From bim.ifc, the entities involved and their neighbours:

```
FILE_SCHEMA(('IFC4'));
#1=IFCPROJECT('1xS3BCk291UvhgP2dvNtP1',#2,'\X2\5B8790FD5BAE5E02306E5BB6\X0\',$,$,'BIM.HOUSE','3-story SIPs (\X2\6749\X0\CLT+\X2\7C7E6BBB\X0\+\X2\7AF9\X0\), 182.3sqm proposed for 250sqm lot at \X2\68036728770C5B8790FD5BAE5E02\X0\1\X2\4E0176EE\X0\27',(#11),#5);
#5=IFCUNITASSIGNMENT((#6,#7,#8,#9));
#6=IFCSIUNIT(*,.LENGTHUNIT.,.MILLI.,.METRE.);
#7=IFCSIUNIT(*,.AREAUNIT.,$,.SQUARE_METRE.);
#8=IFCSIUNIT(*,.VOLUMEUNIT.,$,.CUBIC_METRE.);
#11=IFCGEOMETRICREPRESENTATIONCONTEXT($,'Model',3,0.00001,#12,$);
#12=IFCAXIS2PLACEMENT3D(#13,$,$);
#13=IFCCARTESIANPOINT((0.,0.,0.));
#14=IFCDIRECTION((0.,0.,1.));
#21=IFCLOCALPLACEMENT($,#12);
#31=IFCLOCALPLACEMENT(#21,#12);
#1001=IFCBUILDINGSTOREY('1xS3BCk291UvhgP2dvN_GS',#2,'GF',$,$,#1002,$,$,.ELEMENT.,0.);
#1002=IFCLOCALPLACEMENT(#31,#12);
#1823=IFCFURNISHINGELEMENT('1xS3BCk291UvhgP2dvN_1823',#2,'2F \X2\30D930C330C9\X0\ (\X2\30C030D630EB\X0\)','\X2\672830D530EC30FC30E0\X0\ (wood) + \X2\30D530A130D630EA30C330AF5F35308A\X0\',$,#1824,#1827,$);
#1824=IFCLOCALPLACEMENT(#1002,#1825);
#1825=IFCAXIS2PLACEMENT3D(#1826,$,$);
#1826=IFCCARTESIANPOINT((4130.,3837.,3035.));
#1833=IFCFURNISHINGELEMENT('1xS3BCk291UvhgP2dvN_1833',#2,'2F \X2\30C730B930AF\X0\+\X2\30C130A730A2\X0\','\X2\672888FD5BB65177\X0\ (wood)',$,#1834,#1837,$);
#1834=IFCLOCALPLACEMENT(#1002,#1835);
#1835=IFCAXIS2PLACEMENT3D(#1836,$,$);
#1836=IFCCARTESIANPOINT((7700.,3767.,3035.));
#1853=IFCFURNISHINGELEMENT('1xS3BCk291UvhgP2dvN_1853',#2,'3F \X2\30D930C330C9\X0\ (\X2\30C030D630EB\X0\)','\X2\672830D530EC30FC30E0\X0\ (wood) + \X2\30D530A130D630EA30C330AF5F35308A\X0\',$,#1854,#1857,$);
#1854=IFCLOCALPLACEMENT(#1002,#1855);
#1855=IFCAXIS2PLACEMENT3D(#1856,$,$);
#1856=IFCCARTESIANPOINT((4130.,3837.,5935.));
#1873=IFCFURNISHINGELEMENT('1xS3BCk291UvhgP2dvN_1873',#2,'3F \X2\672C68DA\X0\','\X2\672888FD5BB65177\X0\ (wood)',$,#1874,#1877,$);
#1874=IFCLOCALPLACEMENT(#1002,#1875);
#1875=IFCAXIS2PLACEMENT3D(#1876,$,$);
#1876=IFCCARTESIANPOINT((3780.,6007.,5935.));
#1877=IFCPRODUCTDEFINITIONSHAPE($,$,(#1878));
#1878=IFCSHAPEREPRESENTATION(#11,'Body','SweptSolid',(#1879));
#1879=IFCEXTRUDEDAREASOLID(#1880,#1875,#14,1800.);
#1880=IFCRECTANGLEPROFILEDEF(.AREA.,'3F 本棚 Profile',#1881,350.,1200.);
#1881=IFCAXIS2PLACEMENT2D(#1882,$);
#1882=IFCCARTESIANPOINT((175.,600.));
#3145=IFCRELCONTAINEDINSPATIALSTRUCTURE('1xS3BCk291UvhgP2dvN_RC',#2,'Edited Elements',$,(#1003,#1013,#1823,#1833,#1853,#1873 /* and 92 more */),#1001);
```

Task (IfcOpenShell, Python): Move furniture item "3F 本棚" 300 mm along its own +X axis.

```python
import ifcopenshell
import ifcopenshell.api.geometry
import ifcopenshell.util.placement
import ifcopenshell.util.unit

model = ifcopenshell.open("bim.ifc")
unit_scale = ifcopenshell.util.unit.calculate_unit_scale(model)

item = model.by_id(1873)
matrix = ifcopenshell.util.placement.get_local_placement(item.ObjectPlacement)
matrix[:3, 3] += matrix[:3, 0] * 0.3 / unit_scale
ifcopenshell.api.geometry.edit_object_placement(model, product=item, matrix=matrix, is_si=False)

print(ifcopenshell.util.placement.get_local_placement(item.ObjectPlacement).round(3) + 0.0)

model.write("bim-out.ifc")
```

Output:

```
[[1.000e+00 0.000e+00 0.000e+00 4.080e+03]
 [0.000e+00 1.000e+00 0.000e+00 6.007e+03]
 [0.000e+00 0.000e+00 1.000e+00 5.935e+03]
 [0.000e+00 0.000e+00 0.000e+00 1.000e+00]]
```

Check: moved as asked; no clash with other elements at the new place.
